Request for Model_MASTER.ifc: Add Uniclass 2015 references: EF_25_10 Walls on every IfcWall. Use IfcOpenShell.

First a look at what the model holds.

```python
import ifcopenshell

model = ifcopenshell.open("Model_MASTER.ifc")
print(model.schema)
print("classifications:", [c.Name for c in model.by_type("IfcClassification")])
for ifc_class in ("IfcDoor", "IfcRoof", "IfcStair", "IfcWall", "IfcWindow"):
    print(ifc_class, len(model.by_type(ifc_class)))
```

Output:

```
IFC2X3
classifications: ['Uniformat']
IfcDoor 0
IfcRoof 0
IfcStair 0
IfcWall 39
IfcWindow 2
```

```python
import ifcopenshell
import ifcopenshell.api.classification

model = ifcopenshell.open("Model_MASTER.ifc")

# IFC2X3 requires Source and Edition and has no link from the project to the system.
system = model.create_entity("IfcClassification", Source="NBS", Edition="2015", Name="Uniclass 2015")

codes = {
    "IfcWall": ("EF_25_10", "Walls"),
}
for ifc_class, (code, name) in codes.items():
    products = model.by_type(ifc_class)
    ifcopenshell.api.classification.add_reference(
        model, products=products, classification=system, identification=code, name=name
    )
    print(code, len(products))

model.write("Model_MASTER_rev.ifc")
```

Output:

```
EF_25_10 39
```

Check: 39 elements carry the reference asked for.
